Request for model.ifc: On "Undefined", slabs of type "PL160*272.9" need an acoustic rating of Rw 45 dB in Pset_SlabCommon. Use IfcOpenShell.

First a look at what the model holds.

```python
import ifcopenshell
import ifcopenshell.util.element

model = ifcopenshell.open("model.ifc")
print(model.schema)
storey = next(s for s in model.by_type("IfcBuildingStorey") if s.Name == "Undefined")
slabs = [e for e in ifcopenshell.util.element.get_decomposition(storey) if e.is_a("IfcSlab")]
seen = {}
for e in slabs:
    element_type = ifcopenshell.util.element.get_type(e)
    key = (element_type.Name if element_type != e and element_type else None, ifcopenshell.util.element.get_pset(e, "Pset_SlabCommon", "AcousticRating"))
    seen[key] = seen.get(key, 0) + 1
for (name, value), count in sorted(seen.items(), key=str):
    print(count, "x", name, "|", value)
```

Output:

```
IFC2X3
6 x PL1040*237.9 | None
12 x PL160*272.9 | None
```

```python
import ifcopenshell
import ifcopenshell.api.pset
import ifcopenshell.util.element

model = ifcopenshell.open("model.ifc")

storey = next(s for s in model.by_type("IfcBuildingStorey") if s.Name == "Undefined")
slabs = [e for e in ifcopenshell.util.element.get_decomposition(storey) if e.is_a("IfcSlab")]

count = 0
for e in slabs:
    element_type = ifcopenshell.util.element.get_type(e)
    if element_type in (None, e) or element_type.Name != "PL160*272.9":
        continue
    # add_pset returns the element's existing set when there is one.
    pset = ifcopenshell.api.pset.add_pset(model, product=e, name="Pset_SlabCommon")
    ifcopenshell.api.pset.edit_pset(model, pset=pset, properties={"AcousticRating": "Rw 45 dB"})
    count += 1

print(count, "slabs updated")

model.write("model_updated.ifc")
```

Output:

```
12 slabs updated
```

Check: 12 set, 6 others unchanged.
